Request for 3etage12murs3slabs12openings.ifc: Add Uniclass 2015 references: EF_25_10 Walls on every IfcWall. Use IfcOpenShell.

First a look at what the model holds.

```python
import ifcopenshell

model = ifcopenshell.open("3etage12murs3slabs12openings.ifc")
print(model.schema)
print("classifications:", [c.Name for c in model.by_type("IfcClassification")])
for ifc_class in ("IfcDoor", "IfcRoof", "IfcStair", "IfcWall", "IfcWindow"):
    print(ifc_class, len(model.by_type(ifc_class)))
```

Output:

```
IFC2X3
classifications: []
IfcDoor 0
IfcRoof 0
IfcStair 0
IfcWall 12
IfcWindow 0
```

```python
import ifcopenshell
import ifcopenshell.api.classification

model = ifcopenshell.open("3etage12murs3slabs12openings.ifc")

# IFC2X3 requires Source and Edition and has no link from the project to the system.
system = model.create_entity("IfcClassification", Source="NBS", Edition="2015", Name="Uniclass 2015")

codes = {
    "IfcWall": ("EF_25_10", "Walls"),
}
for ifc_class, (code, name) in codes.items():
    products = model.by_type(ifc_class)
    ifcopenshell.api.classification.add_reference(
        model, products=products, classification=system, identification=code, name=name
    )
    print(code, len(products))

model.write("3etage12murs3slabs12openings-out.ifc")
```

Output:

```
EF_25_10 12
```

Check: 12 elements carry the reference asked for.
